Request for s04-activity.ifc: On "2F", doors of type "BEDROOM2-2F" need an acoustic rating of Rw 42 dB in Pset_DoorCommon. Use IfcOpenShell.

First a look at what the model holds.

```python
import ifcopenshell
import ifcopenshell.util.element

model = ifcopenshell.open("s04-activity.ifc")
print(model.schema)
storey = next(s for s in model.by_type("IfcBuildingStorey") if s.Name == "2F")
doors = [e for e in ifcopenshell.util.element.get_decomposition(storey) if e.is_a("IfcDoor")]
seen = {}
for e in doors:
    element_type = ifcopenshell.util.element.get_type(e)
    key = (element_type.Name if element_type != e and element_type else None, ifcopenshell.util.element.get_pset(e, "Pset_DoorCommon", "AcousticRating"))
    seen[key] = seen.get(key, 0) + 1
for (name, value), count in sorted(seen.items(), key=str):
    print(count, "x", name, "|", value)
```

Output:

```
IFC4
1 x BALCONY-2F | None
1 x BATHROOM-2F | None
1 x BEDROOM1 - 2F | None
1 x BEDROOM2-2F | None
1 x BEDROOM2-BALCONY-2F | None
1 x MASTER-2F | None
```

```python
import ifcopenshell
import ifcopenshell.api.pset
import ifcopenshell.util.element

model = ifcopenshell.open("s04-activity.ifc")

storey = next(s for s in model.by_type("IfcBuildingStorey") if s.Name == "2F")
doors = [e for e in ifcopenshell.util.element.get_decomposition(storey) if e.is_a("IfcDoor")]

count = 0
for e in doors:
    element_type = ifcopenshell.util.element.get_type(e)
    if element_type in (None, e) or element_type.Name != "BEDROOM2-2F":
        continue
    # add_pset returns the element's existing set when there is one.
    pset = ifcopenshell.api.pset.add_pset(model, product=e, name="Pset_DoorCommon")
    ifcopenshell.api.pset.edit_pset(model, pset=pset, properties={"AcousticRating": "Rw 42 dB"})
    count += 1

print(count, "doors updated")

model.write("s04-activity-out.ifc")
```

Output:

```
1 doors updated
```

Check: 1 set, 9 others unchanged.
